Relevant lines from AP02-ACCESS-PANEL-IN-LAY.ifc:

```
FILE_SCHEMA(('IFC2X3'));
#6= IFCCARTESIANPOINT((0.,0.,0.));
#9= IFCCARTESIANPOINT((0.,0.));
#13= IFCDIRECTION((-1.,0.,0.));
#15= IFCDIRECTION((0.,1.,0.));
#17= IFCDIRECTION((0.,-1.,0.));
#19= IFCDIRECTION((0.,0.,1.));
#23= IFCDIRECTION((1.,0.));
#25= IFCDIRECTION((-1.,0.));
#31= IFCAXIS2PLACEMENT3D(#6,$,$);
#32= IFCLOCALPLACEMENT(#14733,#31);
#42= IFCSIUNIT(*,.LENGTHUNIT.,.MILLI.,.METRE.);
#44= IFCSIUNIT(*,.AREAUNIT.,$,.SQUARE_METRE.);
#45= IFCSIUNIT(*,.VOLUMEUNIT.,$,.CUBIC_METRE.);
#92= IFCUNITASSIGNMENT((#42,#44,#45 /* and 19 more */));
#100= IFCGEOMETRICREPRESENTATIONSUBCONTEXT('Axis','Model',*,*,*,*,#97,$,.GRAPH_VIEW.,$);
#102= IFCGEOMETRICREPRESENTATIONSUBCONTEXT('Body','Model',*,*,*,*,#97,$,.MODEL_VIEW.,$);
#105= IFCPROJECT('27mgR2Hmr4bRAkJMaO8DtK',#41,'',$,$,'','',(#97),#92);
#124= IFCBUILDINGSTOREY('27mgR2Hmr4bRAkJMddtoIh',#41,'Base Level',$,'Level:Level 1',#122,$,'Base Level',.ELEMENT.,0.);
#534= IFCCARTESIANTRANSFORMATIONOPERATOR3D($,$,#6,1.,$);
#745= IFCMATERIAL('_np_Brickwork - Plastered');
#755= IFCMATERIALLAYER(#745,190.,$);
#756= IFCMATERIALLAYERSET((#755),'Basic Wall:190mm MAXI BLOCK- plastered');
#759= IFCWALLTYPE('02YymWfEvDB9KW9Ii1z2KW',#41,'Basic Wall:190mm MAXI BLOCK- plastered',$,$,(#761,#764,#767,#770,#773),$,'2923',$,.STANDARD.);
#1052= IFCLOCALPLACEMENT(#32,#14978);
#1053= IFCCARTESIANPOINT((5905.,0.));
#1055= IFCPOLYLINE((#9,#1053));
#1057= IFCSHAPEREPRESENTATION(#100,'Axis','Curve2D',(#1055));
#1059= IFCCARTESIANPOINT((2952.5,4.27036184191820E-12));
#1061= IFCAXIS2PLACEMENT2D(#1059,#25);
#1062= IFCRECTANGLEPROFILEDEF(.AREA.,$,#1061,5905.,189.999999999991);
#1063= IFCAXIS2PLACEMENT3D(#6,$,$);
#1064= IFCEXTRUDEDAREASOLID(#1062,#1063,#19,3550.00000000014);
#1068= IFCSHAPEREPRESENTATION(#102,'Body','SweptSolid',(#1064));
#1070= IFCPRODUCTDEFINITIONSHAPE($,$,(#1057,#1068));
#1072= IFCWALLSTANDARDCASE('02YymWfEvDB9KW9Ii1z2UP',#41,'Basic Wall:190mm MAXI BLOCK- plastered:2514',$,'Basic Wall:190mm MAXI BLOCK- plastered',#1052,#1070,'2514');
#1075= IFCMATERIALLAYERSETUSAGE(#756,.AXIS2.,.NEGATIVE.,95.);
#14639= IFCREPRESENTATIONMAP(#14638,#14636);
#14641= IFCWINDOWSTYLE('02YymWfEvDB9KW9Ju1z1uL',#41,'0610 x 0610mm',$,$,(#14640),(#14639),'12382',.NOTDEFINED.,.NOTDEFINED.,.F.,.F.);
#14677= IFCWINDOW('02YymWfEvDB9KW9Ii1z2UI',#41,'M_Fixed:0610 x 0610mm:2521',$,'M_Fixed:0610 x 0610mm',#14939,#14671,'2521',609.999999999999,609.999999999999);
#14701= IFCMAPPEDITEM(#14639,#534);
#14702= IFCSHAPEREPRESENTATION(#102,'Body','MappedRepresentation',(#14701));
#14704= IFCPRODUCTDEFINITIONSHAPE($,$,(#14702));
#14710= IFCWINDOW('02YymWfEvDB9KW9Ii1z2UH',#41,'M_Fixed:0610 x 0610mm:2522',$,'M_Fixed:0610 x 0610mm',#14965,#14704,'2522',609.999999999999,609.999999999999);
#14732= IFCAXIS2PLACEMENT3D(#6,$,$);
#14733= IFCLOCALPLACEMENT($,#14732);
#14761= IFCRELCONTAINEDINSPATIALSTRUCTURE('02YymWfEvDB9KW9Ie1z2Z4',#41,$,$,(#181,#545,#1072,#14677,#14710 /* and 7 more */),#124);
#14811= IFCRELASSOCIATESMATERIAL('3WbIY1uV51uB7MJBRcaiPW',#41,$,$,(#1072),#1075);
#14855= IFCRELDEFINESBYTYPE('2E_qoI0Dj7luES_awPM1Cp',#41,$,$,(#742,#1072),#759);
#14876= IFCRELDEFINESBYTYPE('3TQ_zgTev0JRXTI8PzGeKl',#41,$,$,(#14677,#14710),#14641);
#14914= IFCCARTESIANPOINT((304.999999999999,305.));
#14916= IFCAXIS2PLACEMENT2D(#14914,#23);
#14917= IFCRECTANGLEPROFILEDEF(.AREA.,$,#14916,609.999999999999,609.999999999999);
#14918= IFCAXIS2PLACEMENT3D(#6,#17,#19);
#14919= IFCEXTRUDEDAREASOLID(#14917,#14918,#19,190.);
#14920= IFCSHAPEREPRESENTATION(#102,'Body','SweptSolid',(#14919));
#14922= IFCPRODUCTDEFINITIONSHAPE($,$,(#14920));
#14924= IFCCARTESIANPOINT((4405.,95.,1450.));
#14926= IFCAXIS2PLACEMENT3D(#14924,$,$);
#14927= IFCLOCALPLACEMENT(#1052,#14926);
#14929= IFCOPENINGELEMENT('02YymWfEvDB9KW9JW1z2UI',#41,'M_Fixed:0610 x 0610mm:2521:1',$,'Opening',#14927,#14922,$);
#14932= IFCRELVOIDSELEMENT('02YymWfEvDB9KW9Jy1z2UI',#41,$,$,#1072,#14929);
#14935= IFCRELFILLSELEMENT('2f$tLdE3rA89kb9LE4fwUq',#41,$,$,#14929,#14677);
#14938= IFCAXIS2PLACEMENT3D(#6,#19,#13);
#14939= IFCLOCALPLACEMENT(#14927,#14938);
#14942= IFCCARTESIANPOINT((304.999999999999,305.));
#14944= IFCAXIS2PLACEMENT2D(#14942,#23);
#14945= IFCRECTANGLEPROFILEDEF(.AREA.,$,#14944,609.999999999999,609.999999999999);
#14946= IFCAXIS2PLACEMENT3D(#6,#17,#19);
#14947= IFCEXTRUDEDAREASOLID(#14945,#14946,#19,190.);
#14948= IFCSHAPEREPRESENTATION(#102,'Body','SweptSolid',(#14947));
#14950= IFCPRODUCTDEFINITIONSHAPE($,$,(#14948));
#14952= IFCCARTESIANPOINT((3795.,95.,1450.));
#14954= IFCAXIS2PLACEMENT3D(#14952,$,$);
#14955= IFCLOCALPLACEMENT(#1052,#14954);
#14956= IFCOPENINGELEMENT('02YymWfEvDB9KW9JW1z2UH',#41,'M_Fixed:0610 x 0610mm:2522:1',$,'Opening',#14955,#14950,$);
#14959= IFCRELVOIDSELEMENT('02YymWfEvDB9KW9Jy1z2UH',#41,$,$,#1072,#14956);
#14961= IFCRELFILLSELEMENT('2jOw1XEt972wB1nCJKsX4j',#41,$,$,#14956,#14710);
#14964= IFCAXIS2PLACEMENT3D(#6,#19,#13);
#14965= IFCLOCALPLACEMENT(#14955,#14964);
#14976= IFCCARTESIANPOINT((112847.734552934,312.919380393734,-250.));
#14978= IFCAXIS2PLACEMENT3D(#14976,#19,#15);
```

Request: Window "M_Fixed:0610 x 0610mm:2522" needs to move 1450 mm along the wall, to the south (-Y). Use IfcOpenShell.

```python
import ifcopenshell
import ifcopenshell.api.geometry
import ifcopenshell.util.placement
import ifcopenshell.util.unit

model = ifcopenshell.open("AP02-ACCESS-PANEL-IN-LAY.ifc")
unit_scale = ifcopenshell.util.unit.calculate_unit_scale(model)

window = model.by_guid("02YymWfEvDB9KW9Ii1z2UH")
opening = window.FillsVoids[0].RelatingOpeningElement
wall = opening.VoidsElements[0].RelatingBuildingElement

wall_matrix = ifcopenshell.util.placement.get_local_placement(wall.ObjectPlacement)
shift = wall_matrix[:3, 0] * -1.45 / unit_scale
before = ifcopenshell.util.placement.get_local_placement(window.ObjectPlacement)[:3, 3].copy()

# The window is placed relative to its opening, so it follows when the opening moves.
matrix = ifcopenshell.util.placement.get_local_placement(opening.ObjectPlacement)
matrix[:3, 3] += shift
ifcopenshell.api.geometry.edit_object_placement(
    model, product=opening, matrix=matrix, is_si=False, should_transform_children=True
)

after = ifcopenshell.util.placement.get_local_placement(window.ObjectPlacement)[:3, 3]
print("window moved by", (after - before).round(3) + 0.0)

model.write("AP02-ACCESS-PANEL-IN-LAY_rev.ifc")
```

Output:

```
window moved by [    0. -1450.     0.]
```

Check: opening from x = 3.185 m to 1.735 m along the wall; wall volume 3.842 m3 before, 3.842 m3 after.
